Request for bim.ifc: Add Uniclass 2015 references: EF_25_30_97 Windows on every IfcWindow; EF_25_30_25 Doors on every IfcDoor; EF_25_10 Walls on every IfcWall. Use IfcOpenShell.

First a look at what the model holds.

```python
import ifcopenshell

model = ifcopenshell.open("bim.ifc")
print(model.schema)
print("classifications:", [c.Name for c in model.by_type("IfcClassification")])
for ifc_class in ("IfcDoor", "IfcRoof", "IfcStair", "IfcWall", "IfcWindow"):
    print(ifc_class, len(model.by_type(ifc_class)))
```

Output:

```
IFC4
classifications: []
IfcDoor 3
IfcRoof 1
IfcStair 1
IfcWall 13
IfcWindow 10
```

```python
import ifcopenshell
import ifcopenshell.api.classification

model = ifcopenshell.open("bim.ifc")

system = ifcopenshell.api.classification.add_classification(model, classification="Uniclass 2015")

codes = {
    "IfcWindow": ("EF_25_30_97", "Windows"),
    "IfcDoor": ("EF_25_30_25", "Doors"),
    "IfcWall": ("EF_25_10", "Walls"),
}
for ifc_class, (code, name) in codes.items():
    products = model.by_type(ifc_class)
    ifcopenshell.api.classification.add_reference(
        model, products=products, classification=system, identification=code, name=name
    )
    print(code, len(products))

model.write("bim_rev.ifc")
```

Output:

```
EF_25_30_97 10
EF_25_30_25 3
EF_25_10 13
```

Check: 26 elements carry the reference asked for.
